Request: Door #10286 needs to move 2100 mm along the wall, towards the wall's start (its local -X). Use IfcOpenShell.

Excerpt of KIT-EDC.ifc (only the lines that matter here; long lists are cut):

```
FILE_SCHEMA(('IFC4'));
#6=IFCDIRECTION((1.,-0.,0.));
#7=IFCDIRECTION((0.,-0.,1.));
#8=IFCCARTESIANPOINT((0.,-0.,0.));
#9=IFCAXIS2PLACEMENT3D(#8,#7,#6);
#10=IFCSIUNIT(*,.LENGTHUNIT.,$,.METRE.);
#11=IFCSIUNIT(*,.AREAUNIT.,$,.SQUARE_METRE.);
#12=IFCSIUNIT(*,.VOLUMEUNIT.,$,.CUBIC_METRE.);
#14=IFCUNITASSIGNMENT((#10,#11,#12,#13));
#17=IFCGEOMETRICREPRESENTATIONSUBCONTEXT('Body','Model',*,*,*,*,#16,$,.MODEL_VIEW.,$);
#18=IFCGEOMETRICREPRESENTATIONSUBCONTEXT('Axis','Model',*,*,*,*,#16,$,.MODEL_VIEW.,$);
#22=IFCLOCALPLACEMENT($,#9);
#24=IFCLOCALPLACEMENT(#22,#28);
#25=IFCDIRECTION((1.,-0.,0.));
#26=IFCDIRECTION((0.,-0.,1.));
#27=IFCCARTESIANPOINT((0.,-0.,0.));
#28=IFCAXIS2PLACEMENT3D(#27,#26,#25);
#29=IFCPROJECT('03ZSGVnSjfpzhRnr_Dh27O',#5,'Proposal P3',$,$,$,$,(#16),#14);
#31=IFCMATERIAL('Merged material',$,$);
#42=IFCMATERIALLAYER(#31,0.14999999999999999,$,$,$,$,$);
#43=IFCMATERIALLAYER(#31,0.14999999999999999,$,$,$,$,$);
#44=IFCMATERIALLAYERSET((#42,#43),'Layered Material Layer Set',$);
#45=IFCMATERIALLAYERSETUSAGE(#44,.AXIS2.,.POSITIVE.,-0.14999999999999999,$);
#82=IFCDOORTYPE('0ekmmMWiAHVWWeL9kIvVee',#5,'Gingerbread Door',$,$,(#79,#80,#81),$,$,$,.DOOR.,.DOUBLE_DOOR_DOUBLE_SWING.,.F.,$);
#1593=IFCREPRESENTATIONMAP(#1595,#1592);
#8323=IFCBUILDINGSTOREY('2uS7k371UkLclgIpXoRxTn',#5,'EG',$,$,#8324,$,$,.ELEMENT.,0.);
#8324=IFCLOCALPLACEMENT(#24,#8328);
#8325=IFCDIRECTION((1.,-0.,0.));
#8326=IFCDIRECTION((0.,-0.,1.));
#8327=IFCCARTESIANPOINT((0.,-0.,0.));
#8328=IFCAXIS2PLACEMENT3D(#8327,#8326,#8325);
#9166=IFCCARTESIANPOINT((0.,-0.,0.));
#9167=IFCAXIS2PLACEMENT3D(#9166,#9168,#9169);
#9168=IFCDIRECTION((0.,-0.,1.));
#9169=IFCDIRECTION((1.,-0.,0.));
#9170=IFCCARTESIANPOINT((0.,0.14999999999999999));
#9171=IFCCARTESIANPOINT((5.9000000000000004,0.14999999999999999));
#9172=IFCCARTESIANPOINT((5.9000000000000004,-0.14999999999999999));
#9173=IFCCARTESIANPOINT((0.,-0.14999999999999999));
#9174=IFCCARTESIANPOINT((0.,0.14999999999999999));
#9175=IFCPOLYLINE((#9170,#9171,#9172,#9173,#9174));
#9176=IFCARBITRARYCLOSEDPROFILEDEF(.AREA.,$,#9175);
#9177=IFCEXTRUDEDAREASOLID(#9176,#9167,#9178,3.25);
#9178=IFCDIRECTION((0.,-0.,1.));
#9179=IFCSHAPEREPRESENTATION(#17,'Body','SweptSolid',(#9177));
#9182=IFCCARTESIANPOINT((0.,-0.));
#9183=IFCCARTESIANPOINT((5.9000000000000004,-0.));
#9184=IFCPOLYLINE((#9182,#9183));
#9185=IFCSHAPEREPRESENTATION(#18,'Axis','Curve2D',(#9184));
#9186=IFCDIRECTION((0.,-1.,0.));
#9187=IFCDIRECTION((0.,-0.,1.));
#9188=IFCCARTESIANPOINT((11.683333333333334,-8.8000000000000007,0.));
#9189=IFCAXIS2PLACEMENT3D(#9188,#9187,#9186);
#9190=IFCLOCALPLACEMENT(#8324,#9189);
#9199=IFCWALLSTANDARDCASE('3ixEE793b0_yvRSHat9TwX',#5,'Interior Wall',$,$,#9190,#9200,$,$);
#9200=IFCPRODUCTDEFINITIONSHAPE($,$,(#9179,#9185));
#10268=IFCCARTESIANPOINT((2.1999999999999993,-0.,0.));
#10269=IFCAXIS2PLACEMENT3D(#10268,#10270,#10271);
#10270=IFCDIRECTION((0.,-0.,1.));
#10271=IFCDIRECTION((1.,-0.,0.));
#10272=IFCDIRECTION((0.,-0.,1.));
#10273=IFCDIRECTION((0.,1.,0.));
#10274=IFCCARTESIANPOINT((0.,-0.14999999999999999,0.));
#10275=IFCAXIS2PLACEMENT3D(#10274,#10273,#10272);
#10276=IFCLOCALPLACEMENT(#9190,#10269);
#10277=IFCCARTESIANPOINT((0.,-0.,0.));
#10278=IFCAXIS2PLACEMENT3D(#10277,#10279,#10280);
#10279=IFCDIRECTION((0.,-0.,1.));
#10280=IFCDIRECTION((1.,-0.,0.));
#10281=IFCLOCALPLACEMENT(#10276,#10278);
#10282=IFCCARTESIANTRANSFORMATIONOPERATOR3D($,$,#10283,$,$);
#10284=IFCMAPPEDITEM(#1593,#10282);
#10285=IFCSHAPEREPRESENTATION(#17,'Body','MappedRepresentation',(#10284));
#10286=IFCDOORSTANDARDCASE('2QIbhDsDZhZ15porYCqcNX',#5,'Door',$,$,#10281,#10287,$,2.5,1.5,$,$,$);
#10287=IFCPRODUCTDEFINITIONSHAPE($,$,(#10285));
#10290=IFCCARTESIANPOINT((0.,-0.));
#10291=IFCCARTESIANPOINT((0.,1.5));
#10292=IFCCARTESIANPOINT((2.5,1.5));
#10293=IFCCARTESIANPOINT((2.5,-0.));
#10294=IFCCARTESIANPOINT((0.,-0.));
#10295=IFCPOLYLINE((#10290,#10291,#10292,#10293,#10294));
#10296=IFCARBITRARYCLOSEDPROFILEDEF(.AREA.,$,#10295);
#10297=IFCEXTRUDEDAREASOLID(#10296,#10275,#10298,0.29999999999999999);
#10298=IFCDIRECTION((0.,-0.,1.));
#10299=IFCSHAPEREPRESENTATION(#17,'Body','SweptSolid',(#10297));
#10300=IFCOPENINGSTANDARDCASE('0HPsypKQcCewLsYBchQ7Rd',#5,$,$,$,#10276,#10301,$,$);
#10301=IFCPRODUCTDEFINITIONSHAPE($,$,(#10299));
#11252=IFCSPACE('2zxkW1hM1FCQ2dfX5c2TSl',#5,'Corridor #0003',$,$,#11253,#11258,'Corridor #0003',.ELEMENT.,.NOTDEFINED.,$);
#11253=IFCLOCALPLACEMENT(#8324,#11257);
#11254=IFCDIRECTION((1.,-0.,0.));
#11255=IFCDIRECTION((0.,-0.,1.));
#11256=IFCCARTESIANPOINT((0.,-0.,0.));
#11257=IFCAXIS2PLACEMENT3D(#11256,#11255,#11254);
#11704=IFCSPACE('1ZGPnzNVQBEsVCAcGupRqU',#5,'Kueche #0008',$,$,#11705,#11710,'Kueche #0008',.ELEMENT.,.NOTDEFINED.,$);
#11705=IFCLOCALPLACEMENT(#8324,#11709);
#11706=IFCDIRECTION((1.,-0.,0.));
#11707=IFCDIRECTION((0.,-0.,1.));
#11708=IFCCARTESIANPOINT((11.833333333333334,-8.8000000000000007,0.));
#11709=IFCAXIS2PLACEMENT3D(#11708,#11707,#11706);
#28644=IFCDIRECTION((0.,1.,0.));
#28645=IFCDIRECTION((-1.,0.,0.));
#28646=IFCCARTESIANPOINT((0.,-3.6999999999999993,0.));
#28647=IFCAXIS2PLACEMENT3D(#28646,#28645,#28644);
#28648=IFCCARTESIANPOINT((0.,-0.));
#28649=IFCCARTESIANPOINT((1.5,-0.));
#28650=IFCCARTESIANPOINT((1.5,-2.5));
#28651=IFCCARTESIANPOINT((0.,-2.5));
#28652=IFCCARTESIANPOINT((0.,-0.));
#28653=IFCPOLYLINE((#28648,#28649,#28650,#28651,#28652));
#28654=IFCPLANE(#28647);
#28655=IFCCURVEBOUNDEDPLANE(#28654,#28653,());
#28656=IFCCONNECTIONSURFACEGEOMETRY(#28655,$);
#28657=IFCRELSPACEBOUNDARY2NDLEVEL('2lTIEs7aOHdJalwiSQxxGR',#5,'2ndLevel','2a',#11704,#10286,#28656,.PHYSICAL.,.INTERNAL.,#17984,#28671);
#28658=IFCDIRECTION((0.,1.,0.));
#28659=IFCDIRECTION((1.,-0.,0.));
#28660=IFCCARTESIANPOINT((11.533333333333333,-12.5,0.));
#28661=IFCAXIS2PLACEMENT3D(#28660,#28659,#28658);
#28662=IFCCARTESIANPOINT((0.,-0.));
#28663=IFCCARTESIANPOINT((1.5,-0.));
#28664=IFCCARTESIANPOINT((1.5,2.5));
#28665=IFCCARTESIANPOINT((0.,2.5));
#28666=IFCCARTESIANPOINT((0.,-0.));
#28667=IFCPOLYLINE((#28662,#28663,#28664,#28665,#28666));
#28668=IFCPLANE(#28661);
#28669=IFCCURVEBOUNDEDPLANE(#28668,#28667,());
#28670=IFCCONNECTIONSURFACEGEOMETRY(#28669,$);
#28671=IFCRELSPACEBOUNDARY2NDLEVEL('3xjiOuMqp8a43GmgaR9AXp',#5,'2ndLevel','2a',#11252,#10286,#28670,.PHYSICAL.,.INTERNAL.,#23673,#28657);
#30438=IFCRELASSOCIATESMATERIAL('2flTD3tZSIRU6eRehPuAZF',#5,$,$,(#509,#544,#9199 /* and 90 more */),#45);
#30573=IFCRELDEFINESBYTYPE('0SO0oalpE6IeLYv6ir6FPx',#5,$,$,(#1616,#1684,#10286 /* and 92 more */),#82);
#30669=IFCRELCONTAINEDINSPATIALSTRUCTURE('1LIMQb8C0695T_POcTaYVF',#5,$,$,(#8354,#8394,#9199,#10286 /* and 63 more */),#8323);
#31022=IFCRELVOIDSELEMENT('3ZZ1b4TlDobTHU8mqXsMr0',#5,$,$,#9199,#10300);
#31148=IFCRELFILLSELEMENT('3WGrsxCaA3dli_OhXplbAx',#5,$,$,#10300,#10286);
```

```python
import numpy as np
import ifcopenshell
import ifcopenshell.api.geometry
import ifcopenshell.util.placement
import ifcopenshell.util.unit

model = ifcopenshell.open("KIT-EDC.ifc")
unit_scale = ifcopenshell.util.unit.calculate_unit_scale(model)

door = model.by_guid("2QIbhDsDZhZ15porYCqcNX")
opening = door.FillsVoids[0].RelatingOpeningElement
wall = opening.VoidsElements[0].RelatingBuildingElement

wall_matrix = ifcopenshell.util.placement.get_local_placement(wall.ObjectPlacement)
shift = wall_matrix[:3, 0] * -2.1 / unit_scale
before = ifcopenshell.util.placement.get_local_placement(door.ObjectPlacement)[:3, 3].copy()

# The door is placed relative to its opening, so it follows when the opening moves.
matrix = ifcopenshell.util.placement.get_local_placement(opening.ObjectPlacement)
matrix[:3, 3] += shift
ifcopenshell.api.geometry.edit_object_placement(
    model, product=opening, matrix=matrix, is_si=False, should_transform_children=True
)

# Space boundary surfaces are stored in each space's coordinates; move them too.
for rel in door.ProvidesBoundaries:
    if not rel.ConnectionGeometry:
        continue
    surface = rel.ConnectionGeometry.SurfaceOnRelatingElement.BasisSurface
    space_matrix = ifcopenshell.util.placement.get_local_placement(rel.RelatingSpace.ObjectPlacement)
    point = np.array(surface.Position.Location.Coordinates) + space_matrix[:3, :3].T @ shift
    surface.Position = model.createIfcAxis2Placement3D(
        model.createIfcCartesianPoint(point.tolist()), surface.Position.Axis, surface.Position.RefDirection
    )

after = ifcopenshell.util.placement.get_local_placement(door.ObjectPlacement)[:3, 3]
print("door moved by", (after - before).round(3) + 0.0)

model.write("KIT-EDC_edited.ifc")
```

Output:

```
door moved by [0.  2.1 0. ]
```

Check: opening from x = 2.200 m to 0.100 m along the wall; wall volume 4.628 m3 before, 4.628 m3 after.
